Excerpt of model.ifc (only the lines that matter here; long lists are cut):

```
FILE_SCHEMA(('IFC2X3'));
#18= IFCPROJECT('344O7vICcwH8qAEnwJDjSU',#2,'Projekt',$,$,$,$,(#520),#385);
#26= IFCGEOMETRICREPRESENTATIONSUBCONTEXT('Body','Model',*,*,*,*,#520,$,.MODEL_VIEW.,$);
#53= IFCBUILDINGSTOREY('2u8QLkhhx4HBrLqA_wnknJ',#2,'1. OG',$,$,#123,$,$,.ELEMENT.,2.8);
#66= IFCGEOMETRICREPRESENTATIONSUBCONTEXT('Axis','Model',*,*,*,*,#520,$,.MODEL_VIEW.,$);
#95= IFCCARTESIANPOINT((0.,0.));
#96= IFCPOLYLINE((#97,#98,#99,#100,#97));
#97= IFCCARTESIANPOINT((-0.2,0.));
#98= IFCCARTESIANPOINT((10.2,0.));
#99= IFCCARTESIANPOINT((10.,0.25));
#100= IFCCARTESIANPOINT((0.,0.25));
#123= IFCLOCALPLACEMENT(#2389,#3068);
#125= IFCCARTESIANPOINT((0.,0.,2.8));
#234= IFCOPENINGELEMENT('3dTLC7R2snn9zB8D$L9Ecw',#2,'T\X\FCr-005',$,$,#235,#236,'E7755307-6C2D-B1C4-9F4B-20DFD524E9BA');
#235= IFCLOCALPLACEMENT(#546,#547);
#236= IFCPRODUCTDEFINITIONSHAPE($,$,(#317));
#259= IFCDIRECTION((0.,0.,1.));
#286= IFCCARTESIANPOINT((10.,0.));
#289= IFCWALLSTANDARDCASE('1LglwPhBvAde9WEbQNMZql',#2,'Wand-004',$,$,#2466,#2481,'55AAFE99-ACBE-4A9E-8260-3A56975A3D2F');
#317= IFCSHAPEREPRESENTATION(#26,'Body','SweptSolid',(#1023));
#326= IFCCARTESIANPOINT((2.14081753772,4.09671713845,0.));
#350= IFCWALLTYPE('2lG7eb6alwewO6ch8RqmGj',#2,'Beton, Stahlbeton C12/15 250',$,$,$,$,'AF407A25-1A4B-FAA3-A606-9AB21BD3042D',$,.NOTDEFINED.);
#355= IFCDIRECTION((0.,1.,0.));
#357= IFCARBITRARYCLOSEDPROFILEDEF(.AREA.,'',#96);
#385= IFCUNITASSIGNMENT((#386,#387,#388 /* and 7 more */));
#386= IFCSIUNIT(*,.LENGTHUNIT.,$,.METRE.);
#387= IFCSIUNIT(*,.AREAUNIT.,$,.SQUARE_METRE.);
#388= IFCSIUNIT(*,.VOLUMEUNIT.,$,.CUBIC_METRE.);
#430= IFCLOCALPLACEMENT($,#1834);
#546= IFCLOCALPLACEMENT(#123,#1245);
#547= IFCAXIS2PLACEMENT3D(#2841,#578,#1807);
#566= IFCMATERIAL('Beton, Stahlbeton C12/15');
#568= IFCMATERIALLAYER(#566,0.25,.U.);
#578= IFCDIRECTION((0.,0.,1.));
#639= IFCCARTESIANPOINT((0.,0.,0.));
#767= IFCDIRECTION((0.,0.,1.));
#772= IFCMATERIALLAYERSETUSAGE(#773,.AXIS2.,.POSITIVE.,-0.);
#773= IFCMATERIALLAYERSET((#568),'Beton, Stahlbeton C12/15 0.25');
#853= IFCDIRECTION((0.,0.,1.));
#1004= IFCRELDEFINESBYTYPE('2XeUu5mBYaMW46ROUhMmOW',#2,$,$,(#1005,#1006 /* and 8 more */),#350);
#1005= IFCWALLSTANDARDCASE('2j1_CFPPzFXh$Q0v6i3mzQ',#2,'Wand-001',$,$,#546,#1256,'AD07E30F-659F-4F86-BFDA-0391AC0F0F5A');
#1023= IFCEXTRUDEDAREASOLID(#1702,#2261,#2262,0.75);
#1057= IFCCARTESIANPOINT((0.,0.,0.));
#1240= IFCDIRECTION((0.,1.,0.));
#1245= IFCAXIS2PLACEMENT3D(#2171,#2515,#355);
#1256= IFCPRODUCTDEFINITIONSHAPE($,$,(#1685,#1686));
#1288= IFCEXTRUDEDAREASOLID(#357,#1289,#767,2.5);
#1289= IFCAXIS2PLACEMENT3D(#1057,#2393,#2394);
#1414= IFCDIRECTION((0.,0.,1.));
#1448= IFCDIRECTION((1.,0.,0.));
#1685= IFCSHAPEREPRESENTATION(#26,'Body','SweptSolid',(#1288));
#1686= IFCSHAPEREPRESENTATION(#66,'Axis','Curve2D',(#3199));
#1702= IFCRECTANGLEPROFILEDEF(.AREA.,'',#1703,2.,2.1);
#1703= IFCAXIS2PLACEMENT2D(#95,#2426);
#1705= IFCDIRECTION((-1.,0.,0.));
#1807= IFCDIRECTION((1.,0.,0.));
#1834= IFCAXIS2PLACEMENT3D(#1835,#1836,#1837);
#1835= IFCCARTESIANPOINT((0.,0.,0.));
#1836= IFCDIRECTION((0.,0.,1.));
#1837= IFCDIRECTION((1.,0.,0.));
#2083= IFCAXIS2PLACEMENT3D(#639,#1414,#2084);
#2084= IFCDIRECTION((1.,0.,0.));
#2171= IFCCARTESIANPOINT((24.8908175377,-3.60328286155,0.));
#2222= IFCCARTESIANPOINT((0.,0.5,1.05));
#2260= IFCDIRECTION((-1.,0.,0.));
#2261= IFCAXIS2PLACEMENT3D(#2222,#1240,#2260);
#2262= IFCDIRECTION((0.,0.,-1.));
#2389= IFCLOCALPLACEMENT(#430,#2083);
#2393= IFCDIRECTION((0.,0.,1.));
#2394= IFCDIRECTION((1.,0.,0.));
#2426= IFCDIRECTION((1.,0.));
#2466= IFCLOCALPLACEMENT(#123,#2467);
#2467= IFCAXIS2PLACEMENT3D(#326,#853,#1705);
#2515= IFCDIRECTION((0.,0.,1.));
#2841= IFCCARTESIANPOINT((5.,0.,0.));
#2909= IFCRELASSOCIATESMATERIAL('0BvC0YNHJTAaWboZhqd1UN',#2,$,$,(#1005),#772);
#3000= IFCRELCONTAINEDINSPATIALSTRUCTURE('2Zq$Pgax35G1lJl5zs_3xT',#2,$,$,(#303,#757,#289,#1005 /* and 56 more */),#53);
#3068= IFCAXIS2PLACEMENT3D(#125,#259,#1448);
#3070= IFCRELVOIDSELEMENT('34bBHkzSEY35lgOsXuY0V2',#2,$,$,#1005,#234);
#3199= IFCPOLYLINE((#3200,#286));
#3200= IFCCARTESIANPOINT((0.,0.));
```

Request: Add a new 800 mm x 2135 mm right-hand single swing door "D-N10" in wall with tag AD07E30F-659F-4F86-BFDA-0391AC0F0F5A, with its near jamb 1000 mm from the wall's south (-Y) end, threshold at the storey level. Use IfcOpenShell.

```python
import numpy as np
import ifcopenshell
import ifcopenshell.api.feature
import ifcopenshell.api.geometry
import ifcopenshell.api.root
import ifcopenshell.api.spatial
import ifcopenshell.api.type
import ifcopenshell.geom
import ifcopenshell.util.element
import ifcopenshell.util.placement
import ifcopenshell.util.representation
import ifcopenshell.util.shape
import ifcopenshell.util.unit

model = ifcopenshell.open("model.ifc")
unit_scale = ifcopenshell.util.unit.calculate_unit_scale(model)
settings = ifcopenshell.geom.settings()


def volume(element):
    """Net volume in cubic metres, openings subtracted."""
    shape = ifcopenshell.geom.create_shape(settings, element)
    return ifcopenshell.util.shape.get_volume(shape.geometry)


wall = model.by_guid("2j1_CFPPzFXh$Q0v6i3mzQ")
storey = ifcopenshell.util.element.get_container(wall, ifc_class="IfcBuildingStorey")
context = ifcopenshell.util.representation.get_context(model, "Model", "Body", "MODEL_VIEW")
before = volume(wall)

width, height, from_end, sill = 0.8, 2.135, 1, 0.0  # metres

# The wall runs along its own X axis, and the end named is its -X end.
wall_shape = ifcopenshell.geom.create_shape(settings, wall)
x, y, z = ifcopenshell.util.shape.get_vertices(wall_shape.geometry).T
start = x.min() + from_end
face, thickness = float(y.min()), float(y.max() - y.min())
wall_matrix = ifcopenshell.util.placement.get_local_placement(wall.ObjectPlacement)
level = ifcopenshell.util.placement.get_local_placement(storey.ObjectPlacement)[2, 3]


def in_wall(x, y):
    """Placement at x, y metres in the wall's axes, at sill height."""
    matrix = wall_matrix.copy()
    matrix[:, 3] = wall_matrix @ np.array([x / unit_scale, y / unit_scale, 0.0, 1.0])
    matrix[2, 3] = level + sill / unit_scale
    return matrix


# Opening: a box that overshoots both wall faces by 50 mm.
opening = ifcopenshell.api.root.create_entity(model, ifc_class="IfcOpeningElement")
box = ifcopenshell.api.geometry.add_wall_representation(
    model, context=context, length=width, height=height, thickness=thickness + 0.1
)
ifcopenshell.api.geometry.assign_representation(model, product=opening, representation=box)
ifcopenshell.api.geometry.edit_object_placement(model, product=opening, matrix=in_wall(start, face - 0.05), is_si=False)
ifcopenshell.api.feature.add_feature(model, feature=opening, element=wall)

door = ifcopenshell.api.root.create_entity(model, ifc_class="IfcDoor", name="D-N10")
door.OverallWidth, door.OverallHeight = width / unit_scale, height / unit_scale
body = ifcopenshell.api.geometry.add_door_representation(
    model,
    context=context,
    overall_width=door.OverallWidth,
    overall_height=door.OverallHeight,
    operation_type="SINGLE_SWING_RIGHT",
    lining_properties={"LiningDepth": thickness / unit_scale, "ThresholdDepth": thickness / unit_scale},
)
ifcopenshell.api.geometry.assign_representation(model, product=door, representation=body)
ifcopenshell.api.spatial.assign_container(model, products=[door], relating_structure=storey)
fills = ifcopenshell.api.feature.add_filling(model, opening=opening, element=door)
fills.OwnerHistory = door.OwnerHistory  # required in IFC2X3

# IFC2X3 keeps the operation on the door style.
style = ifcopenshell.api.root.create_entity(model, ifc_class="IfcDoorStyle", name="D-N10")
style.OperationType, style.ConstructionType = "SINGLE_SWING_RIGHT", "NOTDEFINED"
style.ParameterTakesPrecedence = style.Sizeable = False
ifcopenshell.api.type.assign_type(model, related_objects=[door], relating_type=style)

# The lining spans the wall, so the door starts at the wall face.
ifcopenshell.api.geometry.edit_object_placement(model, product=door, matrix=in_wall(start, face), is_si=False)

after = volume(wall)

print(f"wall volume {before:.3f} -> {after:.3f} m3")

model.write("model_edited.ifc")
```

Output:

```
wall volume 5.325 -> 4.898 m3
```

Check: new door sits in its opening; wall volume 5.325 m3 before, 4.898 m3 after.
